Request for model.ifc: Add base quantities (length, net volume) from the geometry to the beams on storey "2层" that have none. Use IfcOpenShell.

First a look at what the model holds.

```python
import ifcopenshell
import ifcopenshell.util.element
import ifcopenshell.util.unit

model = ifcopenshell.open("model.ifc")
print(model.schema)
for unit_type in ("LENGTHUNIT", "AREAUNIT", "VOLUMEUNIT"):
    print(unit_type, ifcopenshell.util.unit.calculate_unit_scale(model, unit_type))
storey = next(s for s in model.by_type("IfcBuildingStorey") if s.Name == "2层")
beams = [e for e in ifcopenshell.util.element.get_decomposition(storey) if e.is_a("IfcBeam")]
for e in sorted(beams, key=lambda e: e.id()):
    print(e.id(), e.is_a(), e.Name, list(ifcopenshell.util.element.get_psets(e, qtos_only=True)), sep=" | ")
```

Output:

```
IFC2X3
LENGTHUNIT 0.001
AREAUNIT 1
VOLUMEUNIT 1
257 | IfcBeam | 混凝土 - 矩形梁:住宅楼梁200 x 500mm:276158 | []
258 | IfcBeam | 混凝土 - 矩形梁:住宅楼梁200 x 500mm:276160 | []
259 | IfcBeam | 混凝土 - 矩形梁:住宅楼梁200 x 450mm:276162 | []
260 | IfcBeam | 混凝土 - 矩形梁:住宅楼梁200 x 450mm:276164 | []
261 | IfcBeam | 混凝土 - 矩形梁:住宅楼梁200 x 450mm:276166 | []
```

```python
import ifcopenshell
import ifcopenshell.api.pset
import ifcopenshell.geom
import ifcopenshell.util.element
import ifcopenshell.util.shape
import ifcopenshell.util.unit

model = ifcopenshell.open("model.ifc")
unit_scale = ifcopenshell.util.unit.calculate_unit_scale(model)
volume_scale = ifcopenshell.util.unit.calculate_unit_scale(model, "VOLUMEUNIT")
settings = ifcopenshell.geom.settings()

storey = next(s for s in model.by_type("IfcBuildingStorey") if s.Name == "2层")
beams = [e for e in ifcopenshell.util.element.get_decomposition(storey) if e.is_a("IfcBeam")]

for e in sorted(beams, key=lambda e: e.id()):
    if ifcopenshell.util.element.get_psets(e, qtos_only=True, should_inherit=False):
        continue
    # Geometry comes back in metres, in the element's own axes.
    shape = ifcopenshell.geom.create_shape(settings, e)
    values = {
        "Length": ifcopenshell.util.shape.get_max_xyz(shape.geometry) / unit_scale,
        "NetVolume": ifcopenshell.util.shape.get_volume(shape.geometry) / volume_scale,
    }
    qto = ifcopenshell.api.pset.add_qto(model, product=e, name="BaseQuantities")
    ifcopenshell.api.pset.edit_qto(model, qto=qto, properties=values)
    print(e.id(), {k: round(v, 3) for k, v in values.items()})

model.write("model_updated.ifc")
```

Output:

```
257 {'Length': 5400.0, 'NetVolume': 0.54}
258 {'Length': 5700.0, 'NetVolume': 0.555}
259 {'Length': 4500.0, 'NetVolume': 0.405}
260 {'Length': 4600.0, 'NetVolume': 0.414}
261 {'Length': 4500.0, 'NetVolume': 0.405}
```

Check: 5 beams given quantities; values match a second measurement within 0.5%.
